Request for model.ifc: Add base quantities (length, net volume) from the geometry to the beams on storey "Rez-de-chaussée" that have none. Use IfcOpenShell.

First a look at what the model holds.

```python
import ifcopenshell
import ifcopenshell.util.element
import ifcopenshell.util.unit

model = ifcopenshell.open("model.ifc")
print(model.schema)
for unit_type in ("LENGTHUNIT", "AREAUNIT", "VOLUMEUNIT"):
    print(unit_type, ifcopenshell.util.unit.calculate_unit_scale(model, unit_type))
storey = next(s for s in model.by_type("IfcBuildingStorey") if s.Name == "Rez-de-chaussée")
beams = [e for e in ifcopenshell.util.element.get_decomposition(storey) if e.is_a("IfcBeam")]
for e in sorted(beams, key=lambda e: e.id()):
    print(e.id(), e.is_a(), e.Name, list(ifcopenshell.util.element.get_psets(e, qtos_only=True)), sep=" | ")
```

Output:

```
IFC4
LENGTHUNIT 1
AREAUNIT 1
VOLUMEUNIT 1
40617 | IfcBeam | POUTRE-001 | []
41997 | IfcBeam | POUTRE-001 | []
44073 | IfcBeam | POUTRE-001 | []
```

```python
import ifcopenshell
import ifcopenshell.api.pset
import ifcopenshell.geom
import ifcopenshell.util.element
import ifcopenshell.util.shape
import ifcopenshell.util.unit

model = ifcopenshell.open("model.ifc")
unit_scale = ifcopenshell.util.unit.calculate_unit_scale(model)
volume_scale = ifcopenshell.util.unit.calculate_unit_scale(model, "VOLUMEUNIT")
settings = ifcopenshell.geom.settings()

storey = next(s for s in model.by_type("IfcBuildingStorey") if s.Name == "Rez-de-chaussée")
beams = [e for e in ifcopenshell.util.element.get_decomposition(storey) if e.is_a("IfcBeam")]

for e in sorted(beams, key=lambda e: e.id()):
    if ifcopenshell.util.element.get_psets(e, qtos_only=True, should_inherit=False):
        continue
    # Geometry comes back in metres, in the element's own axes.
    shape = ifcopenshell.geom.create_shape(settings, e)
    values = {
        "Length": ifcopenshell.util.shape.get_max_xyz(shape.geometry) / unit_scale,
        "NetVolume": ifcopenshell.util.shape.get_volume(shape.geometry) / volume_scale,
    }
    qto = ifcopenshell.api.pset.add_qto(model, product=e, name="Qto_BeamBaseQuantities")
    ifcopenshell.api.pset.edit_qto(model, qto=qto, properties=values)
    print(e.id(), {k: round(v, 3) for k, v in values.items()})

model.write("model_updated.ifc")
```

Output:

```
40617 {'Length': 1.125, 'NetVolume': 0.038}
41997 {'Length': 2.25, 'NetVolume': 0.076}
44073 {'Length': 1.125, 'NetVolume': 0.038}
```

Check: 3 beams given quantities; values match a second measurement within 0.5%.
